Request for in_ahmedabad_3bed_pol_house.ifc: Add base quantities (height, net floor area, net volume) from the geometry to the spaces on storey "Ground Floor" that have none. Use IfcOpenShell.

First a look at what the model holds.

```python
import ifcopenshell
import ifcopenshell.util.element
import ifcopenshell.util.unit

model = ifcopenshell.open("in_ahmedabad_3bed_pol_house.ifc")
print(model.schema)
for unit_type in ("LENGTHUNIT", "AREAUNIT", "VOLUMEUNIT"):
    print(unit_type, ifcopenshell.util.unit.calculate_unit_scale(model, unit_type))
storey = next(s for s in model.by_type("IfcBuildingStorey") if s.Name == "Ground Floor")
spaces = [e for e in ifcopenshell.util.element.get_decomposition(storey) if e.is_a("IfcSpace")]
for e in sorted(spaces, key=lambda e: e.id()):
    print(e.id(), e.is_a(), e.Name, list(ifcopenshell.util.element.get_psets(e, qtos_only=True)), sep=" | ")
```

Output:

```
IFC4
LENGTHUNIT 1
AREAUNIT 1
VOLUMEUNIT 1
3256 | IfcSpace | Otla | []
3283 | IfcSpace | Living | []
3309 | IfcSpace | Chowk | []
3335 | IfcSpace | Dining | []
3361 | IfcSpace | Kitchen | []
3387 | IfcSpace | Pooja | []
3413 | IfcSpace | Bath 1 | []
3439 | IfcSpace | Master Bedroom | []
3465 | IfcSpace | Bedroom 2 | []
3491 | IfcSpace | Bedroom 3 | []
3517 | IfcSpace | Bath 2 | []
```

```python
import ifcopenshell
import ifcopenshell.api.pset
import ifcopenshell.geom
import ifcopenshell.util.element
import ifcopenshell.util.shape
import ifcopenshell.util.unit

model = ifcopenshell.open("in_ahmedabad_3bed_pol_house.ifc")
unit_scale = ifcopenshell.util.unit.calculate_unit_scale(model)
area_scale = ifcopenshell.util.unit.calculate_unit_scale(model, "AREAUNIT")
volume_scale = ifcopenshell.util.unit.calculate_unit_scale(model, "VOLUMEUNIT")
settings = ifcopenshell.geom.settings()

storey = next(s for s in model.by_type("IfcBuildingStorey") if s.Name == "Ground Floor")
spaces = [e for e in ifcopenshell.util.element.get_decomposition(storey) if e.is_a("IfcSpace")]

for e in sorted(spaces, key=lambda e: e.id()):
    if ifcopenshell.util.element.get_psets(e, qtos_only=True, should_inherit=False):
        continue
    # Geometry comes back in metres, in the element's own axes.
    shape = ifcopenshell.geom.create_shape(settings, e)
    values = {
        "Height": ifcopenshell.util.shape.get_z(shape.geometry) / unit_scale,
        "NetFloorArea": ifcopenshell.util.shape.get_footprint_area(shape.geometry) / area_scale,
        "NetVolume": ifcopenshell.util.shape.get_volume(shape.geometry) / volume_scale,
    }
    qto = ifcopenshell.api.pset.add_qto(model, product=e, name="Qto_SpaceBaseQuantities")
    ifcopenshell.api.pset.edit_qto(model, qto=qto, properties=values)
    print(e.id(), {k: round(v, 3) for k, v in values.items()})

model.write("in_ahmedabad_3bed_pol_house_updated.ifc")
```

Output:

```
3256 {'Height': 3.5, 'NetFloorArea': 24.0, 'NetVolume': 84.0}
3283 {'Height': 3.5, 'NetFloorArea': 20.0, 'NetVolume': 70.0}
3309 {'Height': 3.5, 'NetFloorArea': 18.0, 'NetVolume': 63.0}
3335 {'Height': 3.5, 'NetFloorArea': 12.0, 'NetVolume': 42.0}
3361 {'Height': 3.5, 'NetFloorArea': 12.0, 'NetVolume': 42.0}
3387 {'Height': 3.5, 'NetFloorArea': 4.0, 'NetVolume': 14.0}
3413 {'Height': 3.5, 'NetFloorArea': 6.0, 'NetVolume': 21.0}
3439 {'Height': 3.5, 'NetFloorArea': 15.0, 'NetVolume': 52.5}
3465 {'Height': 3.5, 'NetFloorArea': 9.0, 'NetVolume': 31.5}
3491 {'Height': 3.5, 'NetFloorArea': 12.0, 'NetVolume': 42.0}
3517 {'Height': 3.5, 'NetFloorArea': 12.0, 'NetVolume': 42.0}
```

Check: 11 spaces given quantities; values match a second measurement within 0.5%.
